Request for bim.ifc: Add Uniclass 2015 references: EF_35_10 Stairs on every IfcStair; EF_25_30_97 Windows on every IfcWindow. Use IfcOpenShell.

First a look at what the model holds.

```python
import ifcopenshell

model = ifcopenshell.open("bim.ifc")
print(model.schema)
print("classifications:", [c.Name for c in model.by_type("IfcClassification")])
for ifc_class in ("IfcDoor", "IfcRoof", "IfcStair", "IfcWall", "IfcWindow"):
    print(ifc_class, len(model.by_type(ifc_class)))
```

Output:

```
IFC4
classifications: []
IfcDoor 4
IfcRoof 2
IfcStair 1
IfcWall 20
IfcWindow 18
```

```python
import ifcopenshell
import ifcopenshell.api.classification

model = ifcopenshell.open("bim.ifc")

system = ifcopenshell.api.classification.add_classification(model, classification="Uniclass 2015")

codes = {
    "IfcStair": ("EF_35_10", "Stairs"),
    "IfcWindow": ("EF_25_30_97", "Windows"),
}
for ifc_class, (code, name) in codes.items():
    products = model.by_type(ifc_class)
    ifcopenshell.api.classification.add_reference(
        model, products=products, classification=system, identification=code, name=name
    )
    print(code, len(products))

model.write("bim_edited.ifc")
```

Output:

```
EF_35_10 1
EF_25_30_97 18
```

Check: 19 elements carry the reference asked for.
